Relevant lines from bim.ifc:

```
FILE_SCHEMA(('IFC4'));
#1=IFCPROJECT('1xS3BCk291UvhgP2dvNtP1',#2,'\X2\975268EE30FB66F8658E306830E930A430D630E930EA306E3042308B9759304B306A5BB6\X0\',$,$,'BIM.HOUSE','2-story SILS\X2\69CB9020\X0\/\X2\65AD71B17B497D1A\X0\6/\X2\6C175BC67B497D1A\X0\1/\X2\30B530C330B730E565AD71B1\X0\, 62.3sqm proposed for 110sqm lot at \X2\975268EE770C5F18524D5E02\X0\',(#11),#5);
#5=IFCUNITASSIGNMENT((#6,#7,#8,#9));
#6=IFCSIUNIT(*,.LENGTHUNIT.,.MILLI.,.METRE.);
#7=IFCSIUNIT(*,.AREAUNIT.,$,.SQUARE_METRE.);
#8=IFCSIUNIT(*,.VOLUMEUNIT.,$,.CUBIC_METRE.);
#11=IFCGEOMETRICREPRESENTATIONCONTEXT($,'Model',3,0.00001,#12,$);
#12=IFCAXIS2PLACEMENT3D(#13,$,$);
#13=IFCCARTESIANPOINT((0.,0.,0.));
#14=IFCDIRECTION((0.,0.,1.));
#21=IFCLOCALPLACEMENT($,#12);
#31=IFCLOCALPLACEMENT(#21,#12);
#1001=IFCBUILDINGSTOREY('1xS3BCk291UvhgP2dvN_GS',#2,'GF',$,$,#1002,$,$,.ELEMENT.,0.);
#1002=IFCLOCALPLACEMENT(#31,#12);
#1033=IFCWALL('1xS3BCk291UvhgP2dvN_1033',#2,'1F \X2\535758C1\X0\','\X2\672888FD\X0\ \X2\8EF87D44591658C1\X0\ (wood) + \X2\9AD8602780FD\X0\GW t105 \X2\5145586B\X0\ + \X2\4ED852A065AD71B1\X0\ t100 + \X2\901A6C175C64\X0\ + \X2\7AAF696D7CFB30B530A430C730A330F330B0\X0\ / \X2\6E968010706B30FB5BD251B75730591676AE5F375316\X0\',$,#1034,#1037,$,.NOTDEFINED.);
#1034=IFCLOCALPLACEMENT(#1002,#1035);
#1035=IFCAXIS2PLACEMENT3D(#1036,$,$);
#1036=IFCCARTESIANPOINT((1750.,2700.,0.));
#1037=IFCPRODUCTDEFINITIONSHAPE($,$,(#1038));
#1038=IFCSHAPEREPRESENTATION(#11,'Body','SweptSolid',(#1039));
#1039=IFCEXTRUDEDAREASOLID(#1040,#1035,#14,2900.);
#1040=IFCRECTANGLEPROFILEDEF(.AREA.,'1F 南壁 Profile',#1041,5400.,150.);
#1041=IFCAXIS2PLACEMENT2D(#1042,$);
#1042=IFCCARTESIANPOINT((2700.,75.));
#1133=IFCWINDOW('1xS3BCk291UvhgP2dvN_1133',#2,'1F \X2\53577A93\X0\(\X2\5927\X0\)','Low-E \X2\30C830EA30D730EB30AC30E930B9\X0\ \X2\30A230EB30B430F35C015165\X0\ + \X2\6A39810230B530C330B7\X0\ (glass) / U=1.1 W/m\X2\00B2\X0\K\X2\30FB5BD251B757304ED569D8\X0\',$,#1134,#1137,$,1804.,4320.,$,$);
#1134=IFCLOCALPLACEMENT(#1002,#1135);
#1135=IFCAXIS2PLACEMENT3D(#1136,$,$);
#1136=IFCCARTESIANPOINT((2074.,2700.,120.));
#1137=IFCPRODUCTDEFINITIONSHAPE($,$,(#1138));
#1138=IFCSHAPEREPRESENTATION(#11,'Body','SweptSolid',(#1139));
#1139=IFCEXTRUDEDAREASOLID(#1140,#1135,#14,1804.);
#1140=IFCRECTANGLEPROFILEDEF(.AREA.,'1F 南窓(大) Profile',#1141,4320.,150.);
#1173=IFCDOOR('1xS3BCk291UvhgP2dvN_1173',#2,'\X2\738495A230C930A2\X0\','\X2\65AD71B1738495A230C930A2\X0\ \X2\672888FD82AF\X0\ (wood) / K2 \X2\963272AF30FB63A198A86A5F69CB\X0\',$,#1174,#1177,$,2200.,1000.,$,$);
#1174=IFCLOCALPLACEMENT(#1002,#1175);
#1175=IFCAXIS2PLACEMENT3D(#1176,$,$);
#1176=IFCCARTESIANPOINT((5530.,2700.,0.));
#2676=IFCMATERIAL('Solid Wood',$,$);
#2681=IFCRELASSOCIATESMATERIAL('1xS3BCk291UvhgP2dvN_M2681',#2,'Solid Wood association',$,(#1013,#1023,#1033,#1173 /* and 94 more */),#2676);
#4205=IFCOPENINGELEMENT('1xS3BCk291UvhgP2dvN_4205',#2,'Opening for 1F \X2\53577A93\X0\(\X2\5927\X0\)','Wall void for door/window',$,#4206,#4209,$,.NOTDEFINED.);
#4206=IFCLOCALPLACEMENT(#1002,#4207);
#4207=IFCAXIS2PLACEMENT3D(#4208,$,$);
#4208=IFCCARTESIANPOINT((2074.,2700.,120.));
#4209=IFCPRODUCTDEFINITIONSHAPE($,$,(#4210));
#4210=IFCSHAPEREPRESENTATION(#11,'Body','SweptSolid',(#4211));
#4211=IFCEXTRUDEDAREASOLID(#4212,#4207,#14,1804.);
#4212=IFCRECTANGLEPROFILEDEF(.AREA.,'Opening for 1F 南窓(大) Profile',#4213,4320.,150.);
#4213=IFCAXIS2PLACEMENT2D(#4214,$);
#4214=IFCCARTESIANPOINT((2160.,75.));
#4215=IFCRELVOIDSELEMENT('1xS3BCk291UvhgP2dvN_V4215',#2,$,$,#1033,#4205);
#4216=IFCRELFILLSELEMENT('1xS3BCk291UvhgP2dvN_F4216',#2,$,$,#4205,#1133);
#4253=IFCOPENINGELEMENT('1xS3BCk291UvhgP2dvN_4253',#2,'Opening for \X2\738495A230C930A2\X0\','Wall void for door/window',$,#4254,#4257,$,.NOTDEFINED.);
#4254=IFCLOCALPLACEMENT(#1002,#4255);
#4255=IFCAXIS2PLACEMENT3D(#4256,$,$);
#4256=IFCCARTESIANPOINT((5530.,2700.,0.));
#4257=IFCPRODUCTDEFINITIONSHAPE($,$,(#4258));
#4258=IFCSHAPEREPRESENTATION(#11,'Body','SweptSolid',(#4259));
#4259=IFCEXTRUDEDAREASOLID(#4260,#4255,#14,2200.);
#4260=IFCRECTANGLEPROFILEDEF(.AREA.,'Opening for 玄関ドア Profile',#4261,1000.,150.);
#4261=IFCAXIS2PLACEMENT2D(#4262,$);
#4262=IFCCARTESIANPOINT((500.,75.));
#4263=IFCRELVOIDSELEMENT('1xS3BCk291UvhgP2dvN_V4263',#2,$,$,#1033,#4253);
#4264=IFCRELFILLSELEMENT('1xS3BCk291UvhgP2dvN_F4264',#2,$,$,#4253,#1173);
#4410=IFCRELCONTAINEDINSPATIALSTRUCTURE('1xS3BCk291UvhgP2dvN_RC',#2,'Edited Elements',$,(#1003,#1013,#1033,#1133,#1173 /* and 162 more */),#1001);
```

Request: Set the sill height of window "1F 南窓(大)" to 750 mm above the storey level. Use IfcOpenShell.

```python
import numpy as np
import ifcopenshell
import ifcopenshell.api.geometry
import ifcopenshell.geom
import ifcopenshell.util.element
import ifcopenshell.util.placement
import ifcopenshell.util.shape
import ifcopenshell.util.unit

model = ifcopenshell.open("bim.ifc")
unit_scale = ifcopenshell.util.unit.calculate_unit_scale(model)

window = model.by_guid("1xS3BCk291UvhgP2dvN_1133")
opening = window.FillsVoids[0].RelatingOpeningElement
storey = ifcopenshell.util.element.get_container(window, ifc_class="IfcBuildingStorey")
level = ifcopenshell.util.placement.get_local_placement(storey.ObjectPlacement)[2, 3]

# The opening's origin need not be at the sill, so measure its lowest point.
shape = ifcopenshell.geom.create_shape(ifcopenshell.geom.settings(), opening)
bottom = ifcopenshell.util.shape.get_shape_bottom_elevation(shape, shape.geometry) / unit_scale
dz = level + 750.0 - bottom

shift = np.array([0.0, 0.0, dz])
# The window is not placed relative to its opening, so move both.
for product in (opening, window):
    matrix = ifcopenshell.util.placement.get_local_placement(product.ObjectPlacement)
    matrix[:3, 3] += shift
    ifcopenshell.api.geometry.edit_object_placement(model, product=product, matrix=matrix, is_si=False)

print(f"moved by {dz * unit_scale:+.3f} m")

model.write("bim-out.ifc")
```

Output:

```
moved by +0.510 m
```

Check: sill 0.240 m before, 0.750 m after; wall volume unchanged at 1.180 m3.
